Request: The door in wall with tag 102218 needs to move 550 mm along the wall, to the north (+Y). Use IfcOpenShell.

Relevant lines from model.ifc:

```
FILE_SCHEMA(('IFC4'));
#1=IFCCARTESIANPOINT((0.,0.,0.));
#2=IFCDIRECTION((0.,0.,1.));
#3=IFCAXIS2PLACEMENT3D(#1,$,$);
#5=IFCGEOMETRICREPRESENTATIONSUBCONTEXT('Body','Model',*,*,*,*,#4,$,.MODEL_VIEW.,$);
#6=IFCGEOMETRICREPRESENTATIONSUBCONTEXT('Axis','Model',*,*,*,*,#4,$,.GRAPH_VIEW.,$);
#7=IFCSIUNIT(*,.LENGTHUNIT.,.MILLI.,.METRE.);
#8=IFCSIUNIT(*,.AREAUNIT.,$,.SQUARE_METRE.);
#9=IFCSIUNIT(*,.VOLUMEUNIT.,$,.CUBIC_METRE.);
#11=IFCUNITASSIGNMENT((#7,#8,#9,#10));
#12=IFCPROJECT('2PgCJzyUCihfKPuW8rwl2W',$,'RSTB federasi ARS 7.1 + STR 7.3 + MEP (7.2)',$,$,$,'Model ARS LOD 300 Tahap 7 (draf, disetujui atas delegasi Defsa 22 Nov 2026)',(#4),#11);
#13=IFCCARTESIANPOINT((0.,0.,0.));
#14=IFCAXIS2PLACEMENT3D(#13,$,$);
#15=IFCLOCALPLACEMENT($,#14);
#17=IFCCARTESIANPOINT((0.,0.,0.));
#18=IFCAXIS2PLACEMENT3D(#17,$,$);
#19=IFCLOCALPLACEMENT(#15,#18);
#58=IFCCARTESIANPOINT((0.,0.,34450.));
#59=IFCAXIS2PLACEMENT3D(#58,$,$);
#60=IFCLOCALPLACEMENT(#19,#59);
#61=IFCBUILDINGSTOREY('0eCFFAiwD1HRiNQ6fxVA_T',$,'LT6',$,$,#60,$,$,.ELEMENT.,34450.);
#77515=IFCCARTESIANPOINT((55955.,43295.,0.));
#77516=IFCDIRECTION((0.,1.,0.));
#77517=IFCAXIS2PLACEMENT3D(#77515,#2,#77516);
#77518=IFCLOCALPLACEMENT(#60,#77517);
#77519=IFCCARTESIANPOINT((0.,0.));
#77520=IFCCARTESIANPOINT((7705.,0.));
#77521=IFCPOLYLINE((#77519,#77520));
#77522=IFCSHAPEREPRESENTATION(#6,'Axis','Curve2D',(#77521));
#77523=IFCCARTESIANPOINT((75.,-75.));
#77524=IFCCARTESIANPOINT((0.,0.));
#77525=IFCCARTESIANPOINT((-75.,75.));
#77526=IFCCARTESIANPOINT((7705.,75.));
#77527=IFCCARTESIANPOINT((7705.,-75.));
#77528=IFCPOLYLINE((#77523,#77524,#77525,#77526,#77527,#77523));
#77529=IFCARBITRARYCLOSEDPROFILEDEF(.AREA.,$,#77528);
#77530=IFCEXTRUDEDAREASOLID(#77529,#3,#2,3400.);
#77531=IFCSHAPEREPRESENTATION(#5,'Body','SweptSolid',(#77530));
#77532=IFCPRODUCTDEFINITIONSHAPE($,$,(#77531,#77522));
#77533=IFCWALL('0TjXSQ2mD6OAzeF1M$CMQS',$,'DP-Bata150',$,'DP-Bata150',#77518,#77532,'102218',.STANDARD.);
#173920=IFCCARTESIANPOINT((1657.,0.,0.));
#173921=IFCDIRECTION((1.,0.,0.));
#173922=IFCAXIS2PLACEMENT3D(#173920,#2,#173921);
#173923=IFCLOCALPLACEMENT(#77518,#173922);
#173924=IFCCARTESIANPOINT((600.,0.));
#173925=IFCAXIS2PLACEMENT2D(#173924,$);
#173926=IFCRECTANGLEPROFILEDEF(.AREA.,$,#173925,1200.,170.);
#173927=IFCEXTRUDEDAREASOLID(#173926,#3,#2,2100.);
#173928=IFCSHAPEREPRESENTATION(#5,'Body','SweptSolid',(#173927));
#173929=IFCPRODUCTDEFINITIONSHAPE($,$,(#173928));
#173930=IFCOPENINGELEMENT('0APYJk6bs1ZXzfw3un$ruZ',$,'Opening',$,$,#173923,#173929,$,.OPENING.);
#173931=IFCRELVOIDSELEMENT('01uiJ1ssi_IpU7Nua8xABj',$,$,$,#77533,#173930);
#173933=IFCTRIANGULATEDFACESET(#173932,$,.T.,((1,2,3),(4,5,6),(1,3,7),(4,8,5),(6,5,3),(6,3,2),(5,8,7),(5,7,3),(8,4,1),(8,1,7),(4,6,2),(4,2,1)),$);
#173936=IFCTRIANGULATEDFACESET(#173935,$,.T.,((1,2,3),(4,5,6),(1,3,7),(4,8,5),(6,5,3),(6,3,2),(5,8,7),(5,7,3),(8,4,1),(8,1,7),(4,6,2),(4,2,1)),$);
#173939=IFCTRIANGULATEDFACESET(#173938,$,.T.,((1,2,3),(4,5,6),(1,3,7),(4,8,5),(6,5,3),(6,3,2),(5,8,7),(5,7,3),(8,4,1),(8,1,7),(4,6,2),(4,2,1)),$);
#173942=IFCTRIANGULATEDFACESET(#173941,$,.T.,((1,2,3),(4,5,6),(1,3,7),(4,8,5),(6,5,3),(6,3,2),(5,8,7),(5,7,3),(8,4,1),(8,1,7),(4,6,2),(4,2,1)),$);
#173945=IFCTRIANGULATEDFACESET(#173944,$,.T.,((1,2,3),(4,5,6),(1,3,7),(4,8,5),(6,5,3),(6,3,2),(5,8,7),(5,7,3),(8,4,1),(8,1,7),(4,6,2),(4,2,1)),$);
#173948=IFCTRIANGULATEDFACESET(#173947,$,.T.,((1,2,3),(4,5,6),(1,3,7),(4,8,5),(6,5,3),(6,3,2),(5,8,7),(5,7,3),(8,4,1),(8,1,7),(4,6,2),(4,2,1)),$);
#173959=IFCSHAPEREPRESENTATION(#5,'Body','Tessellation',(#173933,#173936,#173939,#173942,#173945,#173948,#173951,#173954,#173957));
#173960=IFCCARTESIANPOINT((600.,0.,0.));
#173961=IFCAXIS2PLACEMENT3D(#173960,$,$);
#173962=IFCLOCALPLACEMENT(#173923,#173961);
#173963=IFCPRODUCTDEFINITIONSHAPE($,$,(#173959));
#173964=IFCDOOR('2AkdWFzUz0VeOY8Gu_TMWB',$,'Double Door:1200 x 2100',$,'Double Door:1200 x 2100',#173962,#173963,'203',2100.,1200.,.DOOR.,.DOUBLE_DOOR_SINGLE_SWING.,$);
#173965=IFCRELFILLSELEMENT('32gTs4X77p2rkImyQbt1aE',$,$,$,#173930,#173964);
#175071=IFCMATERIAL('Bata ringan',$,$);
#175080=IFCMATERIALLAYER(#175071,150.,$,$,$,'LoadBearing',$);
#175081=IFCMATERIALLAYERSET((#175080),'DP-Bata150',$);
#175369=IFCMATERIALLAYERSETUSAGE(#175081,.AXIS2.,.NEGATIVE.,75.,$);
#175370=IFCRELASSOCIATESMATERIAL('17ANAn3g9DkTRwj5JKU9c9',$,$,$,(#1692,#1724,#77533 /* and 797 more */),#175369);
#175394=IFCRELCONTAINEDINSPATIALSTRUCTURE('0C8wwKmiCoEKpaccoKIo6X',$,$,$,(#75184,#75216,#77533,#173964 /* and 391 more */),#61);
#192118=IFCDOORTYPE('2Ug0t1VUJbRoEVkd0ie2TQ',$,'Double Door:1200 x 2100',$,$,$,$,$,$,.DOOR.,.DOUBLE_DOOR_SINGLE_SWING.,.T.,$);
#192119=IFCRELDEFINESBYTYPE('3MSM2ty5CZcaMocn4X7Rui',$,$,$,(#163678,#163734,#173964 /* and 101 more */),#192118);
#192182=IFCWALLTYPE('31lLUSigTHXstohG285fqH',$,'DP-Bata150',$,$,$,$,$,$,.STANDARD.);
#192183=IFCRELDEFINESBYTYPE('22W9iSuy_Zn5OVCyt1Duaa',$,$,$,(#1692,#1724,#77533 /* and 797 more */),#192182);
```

```python
import ifcopenshell
import ifcopenshell.api.geometry
import ifcopenshell.util.placement

model = ifcopenshell.open("model.ifc")

door = model.by_id(173964)
opening = door.FillsVoids[0].RelatingOpeningElement
wall = opening.VoidsElements[0].RelatingBuildingElement

wall_matrix = ifcopenshell.util.placement.get_local_placement(wall.ObjectPlacement)
shift = wall_matrix[:3, 0] * 550.0
before = ifcopenshell.util.placement.get_local_placement(door.ObjectPlacement)[:3, 3].copy()

# The door is placed relative to its opening, so it follows when the opening moves.
matrix = ifcopenshell.util.placement.get_local_placement(opening.ObjectPlacement)
matrix[:3, 3] += shift
ifcopenshell.api.geometry.edit_object_placement(
    model, product=opening, matrix=matrix, is_si=False, should_transform_children=True
)

after = ifcopenshell.util.placement.get_local_placement(door.ObjectPlacement)[:3, 3]
print("door moved by", (after - before).round(3) + 0.0)

model.write("model_rev.ifc")
```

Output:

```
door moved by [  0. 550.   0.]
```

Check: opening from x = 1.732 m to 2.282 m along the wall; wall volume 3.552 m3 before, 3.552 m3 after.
